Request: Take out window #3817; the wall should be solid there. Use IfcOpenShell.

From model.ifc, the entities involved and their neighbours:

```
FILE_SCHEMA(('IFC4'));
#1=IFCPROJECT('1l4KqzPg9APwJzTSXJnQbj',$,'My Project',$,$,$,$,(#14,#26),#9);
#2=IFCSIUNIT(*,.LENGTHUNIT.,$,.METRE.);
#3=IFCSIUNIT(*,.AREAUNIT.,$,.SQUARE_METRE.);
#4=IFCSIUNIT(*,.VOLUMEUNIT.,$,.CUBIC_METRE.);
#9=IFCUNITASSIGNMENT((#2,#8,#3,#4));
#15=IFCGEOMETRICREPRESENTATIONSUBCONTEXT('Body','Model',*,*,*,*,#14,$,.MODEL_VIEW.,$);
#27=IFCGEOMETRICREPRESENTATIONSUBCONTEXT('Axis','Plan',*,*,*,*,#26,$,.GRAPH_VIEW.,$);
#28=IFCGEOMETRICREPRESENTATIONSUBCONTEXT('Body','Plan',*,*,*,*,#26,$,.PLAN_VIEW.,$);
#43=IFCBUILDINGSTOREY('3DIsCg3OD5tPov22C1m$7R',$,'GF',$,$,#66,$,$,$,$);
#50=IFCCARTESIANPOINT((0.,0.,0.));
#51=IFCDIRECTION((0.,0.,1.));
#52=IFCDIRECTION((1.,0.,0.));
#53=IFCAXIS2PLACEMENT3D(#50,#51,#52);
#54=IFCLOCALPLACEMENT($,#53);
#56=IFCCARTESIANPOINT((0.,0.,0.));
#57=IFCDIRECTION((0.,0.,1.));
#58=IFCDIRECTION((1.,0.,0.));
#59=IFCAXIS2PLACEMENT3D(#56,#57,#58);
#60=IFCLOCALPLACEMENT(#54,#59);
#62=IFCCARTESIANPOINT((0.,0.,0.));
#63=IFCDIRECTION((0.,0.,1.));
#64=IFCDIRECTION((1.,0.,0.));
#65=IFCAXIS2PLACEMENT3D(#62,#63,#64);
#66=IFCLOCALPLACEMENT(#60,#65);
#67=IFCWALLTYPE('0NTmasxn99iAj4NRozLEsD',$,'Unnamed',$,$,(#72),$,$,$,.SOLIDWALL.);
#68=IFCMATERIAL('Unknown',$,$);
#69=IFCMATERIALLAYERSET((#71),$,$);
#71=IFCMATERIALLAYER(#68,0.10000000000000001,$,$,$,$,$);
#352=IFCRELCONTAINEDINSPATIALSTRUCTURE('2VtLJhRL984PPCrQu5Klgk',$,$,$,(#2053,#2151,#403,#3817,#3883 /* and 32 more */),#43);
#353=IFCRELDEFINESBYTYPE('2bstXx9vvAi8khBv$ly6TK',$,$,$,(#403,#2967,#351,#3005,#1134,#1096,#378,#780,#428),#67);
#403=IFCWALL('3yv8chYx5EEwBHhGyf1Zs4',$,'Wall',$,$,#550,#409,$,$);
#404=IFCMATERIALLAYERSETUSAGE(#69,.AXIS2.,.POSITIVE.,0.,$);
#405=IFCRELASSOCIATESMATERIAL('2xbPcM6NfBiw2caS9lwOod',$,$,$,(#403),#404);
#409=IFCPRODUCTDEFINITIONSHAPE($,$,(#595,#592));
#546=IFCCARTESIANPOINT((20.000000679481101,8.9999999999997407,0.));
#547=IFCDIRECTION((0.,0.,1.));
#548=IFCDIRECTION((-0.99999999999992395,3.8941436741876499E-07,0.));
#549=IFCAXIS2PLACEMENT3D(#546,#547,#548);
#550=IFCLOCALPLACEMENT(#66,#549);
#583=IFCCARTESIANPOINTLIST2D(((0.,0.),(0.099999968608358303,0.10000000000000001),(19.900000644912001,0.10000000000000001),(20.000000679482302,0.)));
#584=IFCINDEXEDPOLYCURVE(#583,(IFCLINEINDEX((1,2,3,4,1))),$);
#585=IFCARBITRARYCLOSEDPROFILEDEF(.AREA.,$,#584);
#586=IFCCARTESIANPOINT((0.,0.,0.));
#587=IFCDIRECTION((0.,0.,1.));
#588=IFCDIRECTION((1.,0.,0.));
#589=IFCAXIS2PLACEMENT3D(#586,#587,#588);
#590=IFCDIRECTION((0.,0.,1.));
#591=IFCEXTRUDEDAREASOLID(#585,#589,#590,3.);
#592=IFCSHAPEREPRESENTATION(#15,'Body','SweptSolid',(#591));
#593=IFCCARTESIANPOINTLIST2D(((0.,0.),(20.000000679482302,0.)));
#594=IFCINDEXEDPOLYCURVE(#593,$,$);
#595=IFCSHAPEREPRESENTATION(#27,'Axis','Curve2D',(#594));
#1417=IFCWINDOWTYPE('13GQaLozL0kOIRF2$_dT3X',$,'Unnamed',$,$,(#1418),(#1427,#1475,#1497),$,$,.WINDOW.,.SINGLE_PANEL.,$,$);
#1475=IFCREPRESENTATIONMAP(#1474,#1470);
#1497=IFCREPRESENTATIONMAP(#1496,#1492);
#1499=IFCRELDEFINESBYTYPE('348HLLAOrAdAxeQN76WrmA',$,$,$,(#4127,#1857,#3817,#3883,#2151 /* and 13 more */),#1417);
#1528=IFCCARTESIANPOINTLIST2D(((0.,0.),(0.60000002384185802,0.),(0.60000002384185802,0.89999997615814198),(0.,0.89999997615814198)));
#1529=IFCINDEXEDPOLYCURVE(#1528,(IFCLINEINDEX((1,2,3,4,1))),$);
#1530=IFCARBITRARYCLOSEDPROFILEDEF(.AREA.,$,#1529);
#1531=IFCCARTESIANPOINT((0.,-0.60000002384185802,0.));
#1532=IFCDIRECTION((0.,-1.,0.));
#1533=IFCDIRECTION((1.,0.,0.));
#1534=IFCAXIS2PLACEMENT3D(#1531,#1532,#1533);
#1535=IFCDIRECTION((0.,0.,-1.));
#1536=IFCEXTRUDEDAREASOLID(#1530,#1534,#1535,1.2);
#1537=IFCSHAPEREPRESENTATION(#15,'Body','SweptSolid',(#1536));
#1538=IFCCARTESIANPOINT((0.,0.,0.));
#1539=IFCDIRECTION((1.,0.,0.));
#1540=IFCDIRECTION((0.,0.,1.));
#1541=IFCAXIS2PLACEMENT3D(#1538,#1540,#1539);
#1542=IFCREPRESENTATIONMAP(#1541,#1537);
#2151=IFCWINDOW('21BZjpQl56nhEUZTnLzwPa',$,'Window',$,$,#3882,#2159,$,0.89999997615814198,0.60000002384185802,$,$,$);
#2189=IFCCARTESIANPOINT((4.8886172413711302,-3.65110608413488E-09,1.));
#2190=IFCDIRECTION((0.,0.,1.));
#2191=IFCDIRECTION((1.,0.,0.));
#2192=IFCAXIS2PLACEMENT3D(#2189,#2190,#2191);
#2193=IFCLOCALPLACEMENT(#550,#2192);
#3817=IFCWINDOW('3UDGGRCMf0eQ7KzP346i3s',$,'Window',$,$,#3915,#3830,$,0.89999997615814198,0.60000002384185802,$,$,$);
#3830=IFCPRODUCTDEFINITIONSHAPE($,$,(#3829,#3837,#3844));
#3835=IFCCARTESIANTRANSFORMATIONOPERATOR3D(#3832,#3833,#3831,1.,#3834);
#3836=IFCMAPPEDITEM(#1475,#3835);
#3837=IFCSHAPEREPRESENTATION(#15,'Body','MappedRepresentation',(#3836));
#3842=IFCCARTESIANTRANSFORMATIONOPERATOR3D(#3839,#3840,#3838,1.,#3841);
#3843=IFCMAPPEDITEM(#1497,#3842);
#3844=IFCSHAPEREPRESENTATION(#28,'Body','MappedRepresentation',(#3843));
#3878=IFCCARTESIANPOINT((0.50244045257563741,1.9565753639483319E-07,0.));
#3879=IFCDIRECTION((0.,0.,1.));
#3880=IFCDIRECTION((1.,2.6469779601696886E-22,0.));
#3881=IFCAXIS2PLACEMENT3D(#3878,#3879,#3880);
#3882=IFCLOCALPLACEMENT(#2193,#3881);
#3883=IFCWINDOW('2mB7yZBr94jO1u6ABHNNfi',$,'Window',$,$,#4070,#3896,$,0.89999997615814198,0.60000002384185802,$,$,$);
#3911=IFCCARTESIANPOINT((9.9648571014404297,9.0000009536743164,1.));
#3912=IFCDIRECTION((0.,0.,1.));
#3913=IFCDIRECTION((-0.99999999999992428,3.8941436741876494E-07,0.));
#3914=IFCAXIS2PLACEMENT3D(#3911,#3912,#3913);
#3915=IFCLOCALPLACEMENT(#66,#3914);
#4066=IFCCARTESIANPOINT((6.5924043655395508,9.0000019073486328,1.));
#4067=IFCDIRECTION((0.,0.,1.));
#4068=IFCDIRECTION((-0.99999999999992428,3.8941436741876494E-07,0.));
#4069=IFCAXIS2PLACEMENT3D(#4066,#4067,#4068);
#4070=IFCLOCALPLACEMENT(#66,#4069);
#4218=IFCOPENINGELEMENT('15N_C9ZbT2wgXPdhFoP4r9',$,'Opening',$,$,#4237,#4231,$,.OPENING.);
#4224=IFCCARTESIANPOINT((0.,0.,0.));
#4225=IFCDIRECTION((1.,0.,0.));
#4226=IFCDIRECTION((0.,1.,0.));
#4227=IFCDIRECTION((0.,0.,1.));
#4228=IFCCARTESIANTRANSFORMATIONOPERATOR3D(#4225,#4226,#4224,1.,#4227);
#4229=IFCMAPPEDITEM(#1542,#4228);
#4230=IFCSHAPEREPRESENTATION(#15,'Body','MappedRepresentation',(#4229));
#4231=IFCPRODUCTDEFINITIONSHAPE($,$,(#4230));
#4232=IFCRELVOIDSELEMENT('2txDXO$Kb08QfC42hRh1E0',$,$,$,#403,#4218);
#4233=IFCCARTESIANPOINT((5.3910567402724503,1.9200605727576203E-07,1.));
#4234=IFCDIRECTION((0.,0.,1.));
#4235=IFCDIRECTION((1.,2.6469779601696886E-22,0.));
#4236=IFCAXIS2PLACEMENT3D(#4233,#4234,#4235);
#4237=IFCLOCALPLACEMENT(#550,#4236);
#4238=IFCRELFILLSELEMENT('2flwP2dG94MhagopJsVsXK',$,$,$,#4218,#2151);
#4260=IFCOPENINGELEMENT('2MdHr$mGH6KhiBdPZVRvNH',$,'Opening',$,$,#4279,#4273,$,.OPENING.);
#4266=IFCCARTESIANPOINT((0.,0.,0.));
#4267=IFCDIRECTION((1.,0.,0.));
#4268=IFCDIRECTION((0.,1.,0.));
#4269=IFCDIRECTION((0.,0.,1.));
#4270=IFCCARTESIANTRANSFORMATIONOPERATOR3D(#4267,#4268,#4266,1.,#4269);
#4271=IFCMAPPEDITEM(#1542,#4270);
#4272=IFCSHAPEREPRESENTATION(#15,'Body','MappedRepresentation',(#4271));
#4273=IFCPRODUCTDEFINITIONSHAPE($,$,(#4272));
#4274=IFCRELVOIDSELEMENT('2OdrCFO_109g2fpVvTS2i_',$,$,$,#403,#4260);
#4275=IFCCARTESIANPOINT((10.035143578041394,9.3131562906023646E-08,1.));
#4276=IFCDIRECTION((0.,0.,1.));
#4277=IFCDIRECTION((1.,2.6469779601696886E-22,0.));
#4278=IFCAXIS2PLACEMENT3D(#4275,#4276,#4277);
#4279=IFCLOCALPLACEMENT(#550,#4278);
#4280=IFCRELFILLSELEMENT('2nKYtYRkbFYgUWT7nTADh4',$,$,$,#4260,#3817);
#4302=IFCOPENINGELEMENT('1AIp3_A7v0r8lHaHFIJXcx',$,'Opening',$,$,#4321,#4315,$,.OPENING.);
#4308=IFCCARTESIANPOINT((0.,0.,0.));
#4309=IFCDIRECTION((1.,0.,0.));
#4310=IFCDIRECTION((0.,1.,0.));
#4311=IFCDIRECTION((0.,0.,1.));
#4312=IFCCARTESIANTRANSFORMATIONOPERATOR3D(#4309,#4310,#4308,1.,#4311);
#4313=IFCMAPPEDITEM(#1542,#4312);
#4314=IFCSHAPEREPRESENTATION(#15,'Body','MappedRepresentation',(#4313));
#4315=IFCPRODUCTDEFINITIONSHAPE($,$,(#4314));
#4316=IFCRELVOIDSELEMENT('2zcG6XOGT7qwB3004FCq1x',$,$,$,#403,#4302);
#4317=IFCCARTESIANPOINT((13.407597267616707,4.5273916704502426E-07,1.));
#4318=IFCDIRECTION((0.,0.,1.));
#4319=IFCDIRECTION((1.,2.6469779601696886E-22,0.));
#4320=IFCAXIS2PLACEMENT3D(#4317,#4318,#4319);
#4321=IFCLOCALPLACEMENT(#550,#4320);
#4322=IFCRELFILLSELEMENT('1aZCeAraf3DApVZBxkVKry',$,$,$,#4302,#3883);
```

```python
import ifcopenshell
import ifcopenshell.api.feature
import ifcopenshell.api.root
import ifcopenshell.geom
import ifcopenshell.util.shape

model = ifcopenshell.open("model.ifc")
settings = ifcopenshell.geom.settings()


def volume(element):
    """Net volume in cubic metres, openings subtracted."""
    shape = ifcopenshell.geom.create_shape(settings, element)
    return ifcopenshell.util.shape.get_volume(shape.geometry)


window = model.by_guid("3UDGGRCMf0eQ7KzP346i3s")
opening = window.FillsVoids[0].RelatingOpeningElement
wall = opening.VoidsElements[0].RelatingBuildingElement
before = volume(wall)

ifcopenshell.api.root.remove_product(model, product=window)
ifcopenshell.api.feature.remove_feature(model, feature=opening)

after = volume(wall)

print(f"wall volume {before:.3f} -> {after:.3f} m3")

model.write("model-out.ifc")
```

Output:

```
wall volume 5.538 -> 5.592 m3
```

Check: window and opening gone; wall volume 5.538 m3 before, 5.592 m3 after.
